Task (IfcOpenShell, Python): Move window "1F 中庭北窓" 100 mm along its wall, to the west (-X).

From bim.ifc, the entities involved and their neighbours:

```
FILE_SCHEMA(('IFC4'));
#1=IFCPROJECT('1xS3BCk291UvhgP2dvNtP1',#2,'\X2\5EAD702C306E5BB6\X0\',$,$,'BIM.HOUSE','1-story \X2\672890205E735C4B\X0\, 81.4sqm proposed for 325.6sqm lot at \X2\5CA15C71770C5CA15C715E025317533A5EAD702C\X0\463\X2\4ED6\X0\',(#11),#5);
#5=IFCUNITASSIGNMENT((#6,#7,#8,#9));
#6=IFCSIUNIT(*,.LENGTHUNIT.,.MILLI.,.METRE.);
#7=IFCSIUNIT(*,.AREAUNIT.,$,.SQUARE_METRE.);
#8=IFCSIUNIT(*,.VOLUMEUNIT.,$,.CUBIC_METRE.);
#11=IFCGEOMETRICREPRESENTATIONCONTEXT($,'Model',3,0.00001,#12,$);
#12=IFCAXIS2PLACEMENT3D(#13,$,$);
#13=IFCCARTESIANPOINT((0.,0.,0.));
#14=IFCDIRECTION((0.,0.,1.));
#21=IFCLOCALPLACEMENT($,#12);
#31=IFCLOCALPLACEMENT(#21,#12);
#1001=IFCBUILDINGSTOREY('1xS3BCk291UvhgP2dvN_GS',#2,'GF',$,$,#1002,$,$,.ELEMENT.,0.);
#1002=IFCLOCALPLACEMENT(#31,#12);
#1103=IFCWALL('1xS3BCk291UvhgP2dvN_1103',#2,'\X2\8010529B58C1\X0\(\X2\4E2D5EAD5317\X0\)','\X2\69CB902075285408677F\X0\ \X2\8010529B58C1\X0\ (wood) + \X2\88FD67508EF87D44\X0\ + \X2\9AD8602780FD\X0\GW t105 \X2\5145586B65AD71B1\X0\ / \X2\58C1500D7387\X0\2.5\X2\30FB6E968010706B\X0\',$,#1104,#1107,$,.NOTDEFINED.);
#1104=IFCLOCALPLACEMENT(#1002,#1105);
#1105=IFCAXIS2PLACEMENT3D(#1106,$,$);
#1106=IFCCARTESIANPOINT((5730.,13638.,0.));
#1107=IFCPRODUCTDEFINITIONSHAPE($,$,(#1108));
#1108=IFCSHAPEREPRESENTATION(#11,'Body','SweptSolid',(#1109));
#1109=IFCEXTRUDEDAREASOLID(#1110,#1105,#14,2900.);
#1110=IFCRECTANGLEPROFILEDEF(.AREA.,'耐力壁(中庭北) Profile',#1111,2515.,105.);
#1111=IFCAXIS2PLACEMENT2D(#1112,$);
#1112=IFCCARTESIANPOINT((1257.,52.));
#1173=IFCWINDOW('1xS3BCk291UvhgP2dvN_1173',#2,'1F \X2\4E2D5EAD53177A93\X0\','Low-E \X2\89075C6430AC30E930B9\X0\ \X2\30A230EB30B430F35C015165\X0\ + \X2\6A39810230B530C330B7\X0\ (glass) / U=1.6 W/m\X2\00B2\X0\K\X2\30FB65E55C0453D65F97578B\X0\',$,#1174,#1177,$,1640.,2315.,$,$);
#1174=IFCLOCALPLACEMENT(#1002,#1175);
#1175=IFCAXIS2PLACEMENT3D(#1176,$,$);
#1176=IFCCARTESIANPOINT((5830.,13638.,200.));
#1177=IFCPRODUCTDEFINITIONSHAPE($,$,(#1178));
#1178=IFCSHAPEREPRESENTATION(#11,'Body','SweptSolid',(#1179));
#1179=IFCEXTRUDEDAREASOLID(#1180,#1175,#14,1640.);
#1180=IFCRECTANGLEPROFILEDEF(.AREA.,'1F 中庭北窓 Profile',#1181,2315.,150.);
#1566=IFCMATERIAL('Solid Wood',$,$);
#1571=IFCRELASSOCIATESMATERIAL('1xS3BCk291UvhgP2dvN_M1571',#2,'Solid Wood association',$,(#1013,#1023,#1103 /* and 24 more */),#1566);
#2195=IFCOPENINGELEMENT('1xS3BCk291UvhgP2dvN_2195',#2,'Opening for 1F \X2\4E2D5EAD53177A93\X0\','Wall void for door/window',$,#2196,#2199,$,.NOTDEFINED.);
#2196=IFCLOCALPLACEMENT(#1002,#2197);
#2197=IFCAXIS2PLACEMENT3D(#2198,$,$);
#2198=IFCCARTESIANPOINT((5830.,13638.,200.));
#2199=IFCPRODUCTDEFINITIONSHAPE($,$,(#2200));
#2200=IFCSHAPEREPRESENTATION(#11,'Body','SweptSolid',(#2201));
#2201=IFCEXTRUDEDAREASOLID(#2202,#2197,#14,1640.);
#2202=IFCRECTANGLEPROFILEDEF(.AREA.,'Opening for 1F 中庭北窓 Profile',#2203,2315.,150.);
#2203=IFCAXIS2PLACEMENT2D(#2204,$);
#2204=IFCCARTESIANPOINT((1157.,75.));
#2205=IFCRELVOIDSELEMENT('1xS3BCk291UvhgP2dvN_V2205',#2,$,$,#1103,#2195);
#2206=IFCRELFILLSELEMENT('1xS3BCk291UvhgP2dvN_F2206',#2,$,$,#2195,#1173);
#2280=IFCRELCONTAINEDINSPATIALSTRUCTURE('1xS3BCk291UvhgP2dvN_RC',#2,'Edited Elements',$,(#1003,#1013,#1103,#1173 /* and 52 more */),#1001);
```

```python
import ifcopenshell
import ifcopenshell.api.geometry
import ifcopenshell.util.placement
import ifcopenshell.util.unit

model = ifcopenshell.open("bim.ifc")
unit_scale = ifcopenshell.util.unit.calculate_unit_scale(model)

window = model.by_guid("1xS3BCk291UvhgP2dvN_1173")
opening = window.FillsVoids[0].RelatingOpeningElement
wall = opening.VoidsElements[0].RelatingBuildingElement

wall_matrix = ifcopenshell.util.placement.get_local_placement(wall.ObjectPlacement)
shift = wall_matrix[:3, 0] * -0.1 / unit_scale
before = ifcopenshell.util.placement.get_local_placement(window.ObjectPlacement)[:3, 3].copy()

# The window is not placed relative to its opening, so move both.
for product in (opening, window):
    matrix = ifcopenshell.util.placement.get_local_placement(product.ObjectPlacement)
    matrix[:3, 3] += shift
    ifcopenshell.api.geometry.edit_object_placement(model, product=product, matrix=matrix, is_si=False)

after = ifcopenshell.util.placement.get_local_placement(window.ObjectPlacement)[:3, 3]
print("window moved by", (after - before).round(3) + 0.0)

model.write("bim_rev.ifc")
```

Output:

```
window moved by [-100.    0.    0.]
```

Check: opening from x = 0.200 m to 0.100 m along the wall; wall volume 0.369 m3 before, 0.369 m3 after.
